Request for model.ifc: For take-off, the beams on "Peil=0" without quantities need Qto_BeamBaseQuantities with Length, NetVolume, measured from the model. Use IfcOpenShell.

First a look at what the model holds.

```python
import ifcopenshell
import ifcopenshell.util.element
import ifcopenshell.util.unit

model = ifcopenshell.open("model.ifc")
print(model.schema)
for unit_type in ("LENGTHUNIT", "AREAUNIT", "VOLUMEUNIT"):
    print(unit_type, ifcopenshell.util.unit.calculate_unit_scale(model, unit_type))
storey = next(s for s in model.by_type("IfcBuildingStorey") if s.Name == "Peil=0")
beams = [e for e in ifcopenshell.util.element.get_decomposition(storey) if e.is_a("IfcBeam")]
for e in sorted(beams, key=lambda e: e.id()):
    print(e.id(), e.is_a(), e.Name, list(ifcopenshell.util.element.get_psets(e, qtos_only=True)), sep=" | ")
```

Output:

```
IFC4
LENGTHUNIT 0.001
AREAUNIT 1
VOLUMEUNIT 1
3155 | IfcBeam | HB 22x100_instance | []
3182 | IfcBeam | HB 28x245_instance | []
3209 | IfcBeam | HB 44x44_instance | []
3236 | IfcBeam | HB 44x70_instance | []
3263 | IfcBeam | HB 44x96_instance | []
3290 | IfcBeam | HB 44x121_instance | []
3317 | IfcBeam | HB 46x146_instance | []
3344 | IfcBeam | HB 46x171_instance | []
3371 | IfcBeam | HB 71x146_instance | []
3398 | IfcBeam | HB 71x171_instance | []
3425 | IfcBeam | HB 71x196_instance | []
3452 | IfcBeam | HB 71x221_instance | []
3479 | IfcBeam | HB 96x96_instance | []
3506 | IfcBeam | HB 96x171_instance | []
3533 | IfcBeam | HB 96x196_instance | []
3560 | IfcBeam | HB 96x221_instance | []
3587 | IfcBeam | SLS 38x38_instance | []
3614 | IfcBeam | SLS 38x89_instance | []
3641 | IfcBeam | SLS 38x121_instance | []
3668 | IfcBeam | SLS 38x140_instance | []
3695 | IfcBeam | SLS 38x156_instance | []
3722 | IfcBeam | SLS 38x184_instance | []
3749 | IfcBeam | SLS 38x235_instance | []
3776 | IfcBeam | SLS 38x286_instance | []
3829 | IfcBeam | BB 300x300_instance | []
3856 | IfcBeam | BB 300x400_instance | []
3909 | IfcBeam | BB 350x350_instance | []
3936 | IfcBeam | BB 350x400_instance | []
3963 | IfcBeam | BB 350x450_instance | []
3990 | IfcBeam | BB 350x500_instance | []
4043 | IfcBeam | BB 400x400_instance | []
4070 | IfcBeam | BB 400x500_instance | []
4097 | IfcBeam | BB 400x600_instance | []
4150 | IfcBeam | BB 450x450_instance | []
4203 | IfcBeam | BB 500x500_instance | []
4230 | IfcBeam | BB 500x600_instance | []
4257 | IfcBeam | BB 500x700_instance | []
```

```python
import ifcopenshell
import ifcopenshell.api.pset
import ifcopenshell.geom
import ifcopenshell.util.element
import ifcopenshell.util.shape
import ifcopenshell.util.unit

model = ifcopenshell.open("model.ifc")
unit_scale = ifcopenshell.util.unit.calculate_unit_scale(model)
volume_scale = ifcopenshell.util.unit.calculate_unit_scale(model, "VOLUMEUNIT")
settings = ifcopenshell.geom.settings()

storey = next(s for s in model.by_type("IfcBuildingStorey") if s.Name == "Peil=0")
beams = [e for e in ifcopenshell.util.element.get_decomposition(storey) if e.is_a("IfcBeam")]

for e in sorted(beams, key=lambda e: e.id()):
    if ifcopenshell.util.element.get_psets(e, qtos_only=True, should_inherit=False):
        continue
    # Geometry comes back in metres, in the element's own axes.
    shape = ifcopenshell.geom.create_shape(settings, e)
    values = {
        "Length": ifcopenshell.util.shape.get_max_xyz(shape.geometry) / unit_scale,
        "NetVolume": ifcopenshell.util.shape.get_volume(shape.geometry) / volume_scale,
    }
    qto = ifcopenshell.api.pset.add_qto(model, product=e, name="Qto_BeamBaseQuantities")
    ifcopenshell.api.pset.edit_qto(model, qto=qto, properties=values)
    print(e.id(), {k: round(v, 3) for k, v in values.items()})

model.write("model-out.ifc")
```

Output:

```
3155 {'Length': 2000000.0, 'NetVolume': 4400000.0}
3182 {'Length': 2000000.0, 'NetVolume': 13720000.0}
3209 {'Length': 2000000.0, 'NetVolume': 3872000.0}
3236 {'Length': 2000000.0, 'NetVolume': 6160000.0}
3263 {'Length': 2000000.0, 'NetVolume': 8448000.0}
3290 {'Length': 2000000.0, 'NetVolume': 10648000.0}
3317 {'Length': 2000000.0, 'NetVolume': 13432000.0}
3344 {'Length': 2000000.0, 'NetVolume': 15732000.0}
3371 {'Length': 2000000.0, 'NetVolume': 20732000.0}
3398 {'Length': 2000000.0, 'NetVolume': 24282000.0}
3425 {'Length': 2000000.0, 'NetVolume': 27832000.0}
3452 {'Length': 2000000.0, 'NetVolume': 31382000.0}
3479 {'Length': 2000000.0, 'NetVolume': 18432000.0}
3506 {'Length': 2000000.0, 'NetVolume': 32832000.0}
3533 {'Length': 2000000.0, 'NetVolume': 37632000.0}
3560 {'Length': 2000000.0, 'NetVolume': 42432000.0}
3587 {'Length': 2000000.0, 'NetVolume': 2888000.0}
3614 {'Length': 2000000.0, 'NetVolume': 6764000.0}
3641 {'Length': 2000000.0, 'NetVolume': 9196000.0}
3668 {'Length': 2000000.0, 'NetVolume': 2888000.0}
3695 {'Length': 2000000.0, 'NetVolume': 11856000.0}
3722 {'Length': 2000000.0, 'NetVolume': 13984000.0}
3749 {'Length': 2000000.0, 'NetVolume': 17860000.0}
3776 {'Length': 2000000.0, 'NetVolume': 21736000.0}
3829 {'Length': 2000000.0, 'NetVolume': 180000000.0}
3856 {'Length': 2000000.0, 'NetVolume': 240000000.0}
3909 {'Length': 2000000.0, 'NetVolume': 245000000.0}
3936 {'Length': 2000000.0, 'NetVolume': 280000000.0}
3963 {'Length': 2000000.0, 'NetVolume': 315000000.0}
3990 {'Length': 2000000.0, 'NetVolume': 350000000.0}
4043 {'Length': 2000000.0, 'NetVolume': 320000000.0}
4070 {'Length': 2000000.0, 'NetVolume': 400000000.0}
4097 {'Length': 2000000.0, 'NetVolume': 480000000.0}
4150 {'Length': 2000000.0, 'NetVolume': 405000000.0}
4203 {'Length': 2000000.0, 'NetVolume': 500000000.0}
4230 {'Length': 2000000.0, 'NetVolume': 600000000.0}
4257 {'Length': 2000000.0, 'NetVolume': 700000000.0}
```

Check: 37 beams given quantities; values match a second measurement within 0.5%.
